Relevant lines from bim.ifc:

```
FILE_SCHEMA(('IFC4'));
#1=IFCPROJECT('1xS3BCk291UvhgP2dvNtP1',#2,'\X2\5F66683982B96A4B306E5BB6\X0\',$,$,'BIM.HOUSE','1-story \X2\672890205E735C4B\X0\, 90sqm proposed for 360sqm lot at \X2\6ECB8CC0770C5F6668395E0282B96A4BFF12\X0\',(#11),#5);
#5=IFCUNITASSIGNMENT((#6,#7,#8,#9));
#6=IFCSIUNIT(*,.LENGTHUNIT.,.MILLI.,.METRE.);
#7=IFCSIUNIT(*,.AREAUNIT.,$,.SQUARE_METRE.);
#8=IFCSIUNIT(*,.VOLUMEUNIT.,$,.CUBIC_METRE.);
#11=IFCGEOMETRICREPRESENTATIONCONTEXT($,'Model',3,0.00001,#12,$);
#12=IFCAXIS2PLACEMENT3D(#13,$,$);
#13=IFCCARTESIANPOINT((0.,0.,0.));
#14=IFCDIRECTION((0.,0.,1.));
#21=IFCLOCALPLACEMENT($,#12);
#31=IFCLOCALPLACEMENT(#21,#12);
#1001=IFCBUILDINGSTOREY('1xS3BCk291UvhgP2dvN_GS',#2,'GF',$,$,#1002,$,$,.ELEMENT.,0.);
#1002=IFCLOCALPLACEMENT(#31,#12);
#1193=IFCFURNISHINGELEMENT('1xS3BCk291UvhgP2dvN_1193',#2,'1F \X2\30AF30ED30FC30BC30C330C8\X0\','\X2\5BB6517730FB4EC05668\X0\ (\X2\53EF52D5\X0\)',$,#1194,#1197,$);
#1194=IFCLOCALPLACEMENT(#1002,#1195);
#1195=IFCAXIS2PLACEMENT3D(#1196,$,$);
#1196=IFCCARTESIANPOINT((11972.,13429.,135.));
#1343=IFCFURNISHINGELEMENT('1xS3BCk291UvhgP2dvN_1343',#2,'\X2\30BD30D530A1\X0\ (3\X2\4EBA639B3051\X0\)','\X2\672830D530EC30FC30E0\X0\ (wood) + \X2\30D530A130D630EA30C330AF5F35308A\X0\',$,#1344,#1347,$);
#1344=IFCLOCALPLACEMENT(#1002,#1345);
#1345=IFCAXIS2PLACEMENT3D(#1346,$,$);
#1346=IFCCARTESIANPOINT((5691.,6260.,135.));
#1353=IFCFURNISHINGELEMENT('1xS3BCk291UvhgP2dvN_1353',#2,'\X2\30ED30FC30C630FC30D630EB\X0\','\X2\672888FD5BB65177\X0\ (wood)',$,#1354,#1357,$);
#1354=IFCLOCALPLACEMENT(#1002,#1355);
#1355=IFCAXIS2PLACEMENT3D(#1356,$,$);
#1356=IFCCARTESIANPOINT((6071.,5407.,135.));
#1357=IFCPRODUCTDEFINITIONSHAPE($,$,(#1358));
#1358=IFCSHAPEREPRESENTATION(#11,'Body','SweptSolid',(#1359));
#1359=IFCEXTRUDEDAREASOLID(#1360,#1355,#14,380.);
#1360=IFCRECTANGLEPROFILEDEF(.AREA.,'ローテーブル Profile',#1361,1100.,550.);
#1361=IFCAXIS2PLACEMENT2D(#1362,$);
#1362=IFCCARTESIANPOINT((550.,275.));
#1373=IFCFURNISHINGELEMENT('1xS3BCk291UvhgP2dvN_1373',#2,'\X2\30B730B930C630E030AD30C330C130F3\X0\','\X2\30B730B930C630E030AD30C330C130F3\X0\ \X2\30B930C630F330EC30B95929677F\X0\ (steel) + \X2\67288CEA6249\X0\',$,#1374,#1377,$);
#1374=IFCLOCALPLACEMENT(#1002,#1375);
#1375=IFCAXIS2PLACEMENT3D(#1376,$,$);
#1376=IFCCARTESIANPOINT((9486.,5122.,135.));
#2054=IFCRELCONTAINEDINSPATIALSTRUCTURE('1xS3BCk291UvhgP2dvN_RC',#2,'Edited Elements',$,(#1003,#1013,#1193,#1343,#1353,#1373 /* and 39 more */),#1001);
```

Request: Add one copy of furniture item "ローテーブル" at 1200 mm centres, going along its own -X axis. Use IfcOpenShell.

```python
import ifcopenshell
import ifcopenshell.api.geometry
import ifcopenshell.api.root
import ifcopenshell.util.element
import ifcopenshell.util.placement

model = ifcopenshell.open("bim.ifc")


def reuse_history(source, copy):
    """copy_class also copies each property set's owner history, people and application; keep the originals."""
    for rel in copy.IsDefinedBy:
        if rel.is_a("IfcRelDefinesByProperties") and (history := rel.RelatingPropertyDefinition.OwnerHistory):
            rel.RelatingPropertyDefinition.OwnerHistory = source.OwnerHistory
            ifcopenshell.util.element.remove_deep2(model, history)


source = model.by_id(1353)
base = ifcopenshell.util.placement.get_local_placement(source.ObjectPlacement)
step = -base[:3, 0] * 1200.0

for i in range(1, 2):
    copy = ifcopenshell.api.root.copy_class(model, product=source)
    copy.Representation = ifcopenshell.util.element.copy_deep(
        model, source.Representation, exclude=["IfcGeometricRepresentationContext", "IfcRepresentationMap"]
    )
    reuse_history(source, copy)
    matrix = base.copy()
    matrix[:3, 3] += i * step
    print("added at", matrix[:3, 3].round(3) + 0.0)
    ifcopenshell.api.geometry.edit_object_placement(model, product=copy, matrix=matrix, is_si=False)

model.write("bim-out.ifc")
```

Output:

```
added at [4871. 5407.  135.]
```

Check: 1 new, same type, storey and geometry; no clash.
